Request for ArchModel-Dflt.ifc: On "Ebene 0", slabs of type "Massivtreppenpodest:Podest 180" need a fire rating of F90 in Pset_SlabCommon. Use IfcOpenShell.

First a look at what the model holds.

```python
import ifcopenshell
import ifcopenshell.util.element

model = ifcopenshell.open("ArchModel-Dflt.ifc")
print(model.schema)
storey = next(s for s in model.by_type("IfcBuildingStorey") if s.Name == "Ebene 0")
slabs = [e for e in ifcopenshell.util.element.get_decomposition(storey) if e.is_a("IfcSlab")]
seen = {}
for e in slabs:
    element_type = ifcopenshell.util.element.get_type(e)
    key = (element_type.Name if element_type != e and element_type else None, ifcopenshell.util.element.get_pset(e, "Pset_SlabCommon", "FireRating"))
    seen[key] = seen.get(key, 0) + 1
for (name, value), count in sorted(seen.items(), key=str):
    print(count, "x", name, "|", value)
```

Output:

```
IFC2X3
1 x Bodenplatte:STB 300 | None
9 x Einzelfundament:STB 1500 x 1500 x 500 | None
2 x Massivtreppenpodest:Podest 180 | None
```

```python
import ifcopenshell
import ifcopenshell.api.pset
import ifcopenshell.util.element

model = ifcopenshell.open("ArchModel-Dflt.ifc")

storey = next(s for s in model.by_type("IfcBuildingStorey") if s.Name == "Ebene 0")
slabs = [e for e in ifcopenshell.util.element.get_decomposition(storey) if e.is_a("IfcSlab")]

count = 0
for e in slabs:
    element_type = ifcopenshell.util.element.get_type(e)
    if element_type in (None, e) or element_type.Name != "Massivtreppenpodest:Podest 180":
        continue
    # add_pset returns the element's existing set when there is one.
    pset = ifcopenshell.api.pset.add_pset(model, product=e, name="Pset_SlabCommon")
    ifcopenshell.api.pset.edit_pset(model, pset=pset, properties={"FireRating": "F90"})
    count += 1

print(count, "slabs updated")

model.write("ArchModel-Dflt_updated.ifc")
```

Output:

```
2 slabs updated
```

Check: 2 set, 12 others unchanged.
